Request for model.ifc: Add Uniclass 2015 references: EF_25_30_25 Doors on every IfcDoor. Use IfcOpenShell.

First a look at what the model holds.

```python
import ifcopenshell

model = ifcopenshell.open("model.ifc")
print(model.schema)
print("classifications:", [c.Name for c in model.by_type("IfcClassification")])
for ifc_class in ("IfcDoor", "IfcRoof", "IfcStair", "IfcWall", "IfcWindow"):
    print(ifc_class, len(model.by_type(ifc_class)))
```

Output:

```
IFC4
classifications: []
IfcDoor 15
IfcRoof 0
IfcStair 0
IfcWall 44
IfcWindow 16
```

```python
import ifcopenshell
import ifcopenshell.api.classification

model = ifcopenshell.open("model.ifc")

system = ifcopenshell.api.classification.add_classification(model, classification="Uniclass 2015")

codes = {
    "IfcDoor": ("EF_25_30_25", "Doors"),
}
for ifc_class, (code, name) in codes.items():
    products = model.by_type(ifc_class)
    ifcopenshell.api.classification.add_reference(
        model, products=products, classification=system, identification=code, name=name
    )
    print(code, len(products))

model.write("model_rev.ifc")
```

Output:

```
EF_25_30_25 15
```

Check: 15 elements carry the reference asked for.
